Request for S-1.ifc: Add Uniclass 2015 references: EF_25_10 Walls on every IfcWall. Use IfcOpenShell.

First a look at what the model holds.

```python
import ifcopenshell

model = ifcopenshell.open("S-1.ifc")
print(model.schema)
print("classifications:", [c.Name for c in model.by_type("IfcClassification")])
for ifc_class in ("IfcDoor", "IfcRoof", "IfcStair", "IfcWall", "IfcWindow"):
    print(ifc_class, len(model.by_type(ifc_class)))
```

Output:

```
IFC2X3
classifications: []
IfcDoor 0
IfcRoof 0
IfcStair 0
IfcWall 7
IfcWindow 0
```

```python
import ifcopenshell
import ifcopenshell.api.classification

model = ifcopenshell.open("S-1.ifc")

# IFC2X3 requires Source and Edition and has no link from the project to the system.
system = model.create_entity("IfcClassification", Source="NBS", Edition="2015", Name="Uniclass 2015")

codes = {
    "IfcWall": ("EF_25_10", "Walls"),
}
for ifc_class, (code, name) in codes.items():
    products = model.by_type(ifc_class)
    ifcopenshell.api.classification.add_reference(
        model, products=products, classification=system, identification=code, name=name
    )
    print(code, len(products))

model.write("S-1_v2.ifc")
```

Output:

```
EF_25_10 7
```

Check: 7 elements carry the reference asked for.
